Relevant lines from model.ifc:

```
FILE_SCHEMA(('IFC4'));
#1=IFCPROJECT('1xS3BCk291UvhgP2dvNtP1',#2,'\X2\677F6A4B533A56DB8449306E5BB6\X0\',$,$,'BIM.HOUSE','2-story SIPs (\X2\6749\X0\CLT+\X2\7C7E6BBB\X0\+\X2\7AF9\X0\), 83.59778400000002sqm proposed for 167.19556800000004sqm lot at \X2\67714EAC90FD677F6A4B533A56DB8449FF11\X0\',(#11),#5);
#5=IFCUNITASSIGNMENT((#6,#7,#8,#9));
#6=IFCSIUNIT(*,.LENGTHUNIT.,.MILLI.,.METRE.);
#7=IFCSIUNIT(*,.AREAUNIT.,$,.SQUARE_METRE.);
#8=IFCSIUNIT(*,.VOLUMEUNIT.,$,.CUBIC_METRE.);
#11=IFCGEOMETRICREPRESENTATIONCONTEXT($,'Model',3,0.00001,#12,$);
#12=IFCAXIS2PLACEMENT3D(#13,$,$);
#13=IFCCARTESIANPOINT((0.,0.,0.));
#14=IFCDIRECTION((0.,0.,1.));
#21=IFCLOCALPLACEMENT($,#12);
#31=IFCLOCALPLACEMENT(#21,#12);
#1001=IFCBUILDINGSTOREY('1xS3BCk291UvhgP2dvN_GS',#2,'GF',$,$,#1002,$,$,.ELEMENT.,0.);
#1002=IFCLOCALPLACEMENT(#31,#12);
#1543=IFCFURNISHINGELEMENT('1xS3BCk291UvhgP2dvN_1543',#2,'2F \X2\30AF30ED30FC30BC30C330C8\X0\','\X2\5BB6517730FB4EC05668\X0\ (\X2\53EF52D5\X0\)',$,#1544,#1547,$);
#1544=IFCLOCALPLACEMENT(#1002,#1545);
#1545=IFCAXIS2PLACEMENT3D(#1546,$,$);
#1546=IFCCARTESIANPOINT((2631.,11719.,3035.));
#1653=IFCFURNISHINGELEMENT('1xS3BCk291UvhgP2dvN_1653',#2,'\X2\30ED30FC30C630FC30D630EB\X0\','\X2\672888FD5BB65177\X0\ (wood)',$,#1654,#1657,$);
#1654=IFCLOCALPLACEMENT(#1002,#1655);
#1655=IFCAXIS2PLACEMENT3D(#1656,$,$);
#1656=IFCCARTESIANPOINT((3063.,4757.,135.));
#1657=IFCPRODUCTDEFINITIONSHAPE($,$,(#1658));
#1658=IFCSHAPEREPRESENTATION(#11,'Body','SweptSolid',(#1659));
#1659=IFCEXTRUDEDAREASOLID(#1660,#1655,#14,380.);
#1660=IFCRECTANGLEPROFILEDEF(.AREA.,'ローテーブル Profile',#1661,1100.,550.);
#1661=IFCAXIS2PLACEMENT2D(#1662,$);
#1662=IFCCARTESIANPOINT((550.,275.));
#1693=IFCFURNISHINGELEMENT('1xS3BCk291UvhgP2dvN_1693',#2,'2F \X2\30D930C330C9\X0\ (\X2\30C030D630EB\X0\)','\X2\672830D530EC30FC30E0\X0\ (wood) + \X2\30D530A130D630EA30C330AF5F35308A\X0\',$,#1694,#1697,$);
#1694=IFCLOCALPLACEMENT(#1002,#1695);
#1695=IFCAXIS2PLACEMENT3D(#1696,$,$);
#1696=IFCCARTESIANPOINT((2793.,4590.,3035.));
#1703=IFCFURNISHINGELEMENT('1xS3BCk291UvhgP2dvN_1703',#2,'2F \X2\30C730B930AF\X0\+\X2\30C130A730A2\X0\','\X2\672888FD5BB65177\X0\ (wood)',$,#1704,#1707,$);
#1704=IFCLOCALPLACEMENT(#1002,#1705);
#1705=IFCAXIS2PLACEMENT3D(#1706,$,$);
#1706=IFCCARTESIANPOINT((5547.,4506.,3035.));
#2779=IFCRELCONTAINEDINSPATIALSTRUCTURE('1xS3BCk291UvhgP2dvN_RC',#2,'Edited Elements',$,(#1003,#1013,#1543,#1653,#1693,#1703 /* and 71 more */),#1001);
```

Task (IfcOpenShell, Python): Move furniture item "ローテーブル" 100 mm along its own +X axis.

```python
import ifcopenshell
import ifcopenshell.api.geometry
import ifcopenshell.util.placement

model = ifcopenshell.open("model.ifc")

item = model.by_id(1653)
matrix = ifcopenshell.util.placement.get_local_placement(item.ObjectPlacement)
matrix[:3, 3] += matrix[:3, 0] * 100.0
ifcopenshell.api.geometry.edit_object_placement(model, product=item, matrix=matrix, is_si=False)

print(ifcopenshell.util.placement.get_local_placement(item.ObjectPlacement).round(3) + 0.0)

model.write("model_rev.ifc")
```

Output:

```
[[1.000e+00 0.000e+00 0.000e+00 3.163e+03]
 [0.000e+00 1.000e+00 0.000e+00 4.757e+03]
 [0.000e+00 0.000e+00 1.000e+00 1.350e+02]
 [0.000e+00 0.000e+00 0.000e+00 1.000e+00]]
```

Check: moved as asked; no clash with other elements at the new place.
